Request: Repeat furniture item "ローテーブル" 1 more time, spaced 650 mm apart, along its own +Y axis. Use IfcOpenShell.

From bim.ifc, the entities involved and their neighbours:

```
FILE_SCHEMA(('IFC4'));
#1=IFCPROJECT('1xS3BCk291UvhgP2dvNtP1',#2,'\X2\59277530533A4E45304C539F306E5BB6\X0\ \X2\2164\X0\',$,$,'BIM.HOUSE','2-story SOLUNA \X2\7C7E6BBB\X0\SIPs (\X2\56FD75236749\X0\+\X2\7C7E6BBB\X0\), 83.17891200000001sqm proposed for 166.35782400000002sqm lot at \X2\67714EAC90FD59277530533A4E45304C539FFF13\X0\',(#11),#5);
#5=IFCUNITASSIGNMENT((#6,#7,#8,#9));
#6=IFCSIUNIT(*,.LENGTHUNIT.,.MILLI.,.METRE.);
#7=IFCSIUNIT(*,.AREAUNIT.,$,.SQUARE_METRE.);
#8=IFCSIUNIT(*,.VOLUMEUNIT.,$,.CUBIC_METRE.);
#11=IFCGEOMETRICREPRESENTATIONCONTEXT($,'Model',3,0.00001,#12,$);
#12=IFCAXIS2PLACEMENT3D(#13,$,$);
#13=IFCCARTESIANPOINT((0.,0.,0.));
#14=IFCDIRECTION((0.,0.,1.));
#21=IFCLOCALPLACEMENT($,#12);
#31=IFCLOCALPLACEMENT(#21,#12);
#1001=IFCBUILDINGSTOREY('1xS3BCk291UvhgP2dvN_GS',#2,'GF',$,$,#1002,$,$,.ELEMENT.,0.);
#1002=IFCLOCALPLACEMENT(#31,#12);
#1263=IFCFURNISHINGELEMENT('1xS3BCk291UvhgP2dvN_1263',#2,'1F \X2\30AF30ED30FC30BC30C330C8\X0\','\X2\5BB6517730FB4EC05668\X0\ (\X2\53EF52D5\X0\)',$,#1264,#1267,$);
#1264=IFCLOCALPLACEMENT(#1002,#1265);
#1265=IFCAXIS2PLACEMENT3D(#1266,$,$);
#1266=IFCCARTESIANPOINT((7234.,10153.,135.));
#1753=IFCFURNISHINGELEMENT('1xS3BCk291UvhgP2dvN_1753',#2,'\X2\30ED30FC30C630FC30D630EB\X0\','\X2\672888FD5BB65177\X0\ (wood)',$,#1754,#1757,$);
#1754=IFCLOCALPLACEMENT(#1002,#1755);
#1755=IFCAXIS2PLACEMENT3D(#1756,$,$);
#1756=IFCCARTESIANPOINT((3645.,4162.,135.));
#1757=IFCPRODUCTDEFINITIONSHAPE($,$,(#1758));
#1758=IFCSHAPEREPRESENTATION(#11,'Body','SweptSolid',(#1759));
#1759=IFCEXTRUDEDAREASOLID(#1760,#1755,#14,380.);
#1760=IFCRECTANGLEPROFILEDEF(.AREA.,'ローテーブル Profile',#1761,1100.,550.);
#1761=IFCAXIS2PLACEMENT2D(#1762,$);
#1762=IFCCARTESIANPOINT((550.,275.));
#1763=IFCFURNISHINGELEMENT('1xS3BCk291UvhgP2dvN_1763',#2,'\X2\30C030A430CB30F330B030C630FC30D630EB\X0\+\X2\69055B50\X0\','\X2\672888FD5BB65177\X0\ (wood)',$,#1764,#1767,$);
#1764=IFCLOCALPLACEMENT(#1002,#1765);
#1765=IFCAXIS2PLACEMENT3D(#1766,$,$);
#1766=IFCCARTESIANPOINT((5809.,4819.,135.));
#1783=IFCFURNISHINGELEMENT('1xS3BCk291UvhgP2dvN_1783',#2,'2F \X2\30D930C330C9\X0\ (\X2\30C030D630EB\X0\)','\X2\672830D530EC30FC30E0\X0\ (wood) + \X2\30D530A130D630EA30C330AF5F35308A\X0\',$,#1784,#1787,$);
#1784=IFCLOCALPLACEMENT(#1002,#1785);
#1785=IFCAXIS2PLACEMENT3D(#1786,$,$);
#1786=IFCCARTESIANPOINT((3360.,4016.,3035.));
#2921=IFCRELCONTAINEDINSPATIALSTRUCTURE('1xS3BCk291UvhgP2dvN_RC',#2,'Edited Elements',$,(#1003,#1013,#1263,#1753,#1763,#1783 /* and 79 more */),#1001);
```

```python
import ifcopenshell
import ifcopenshell.api.geometry
import ifcopenshell.api.root
import ifcopenshell.util.element
import ifcopenshell.util.placement

model = ifcopenshell.open("bim.ifc")


def reuse_history(source, copy):
    """copy_class also copies each property set's owner history, people and application; keep the originals."""
    for rel in copy.IsDefinedBy:
        if rel.is_a("IfcRelDefinesByProperties") and (history := rel.RelatingPropertyDefinition.OwnerHistory):
            rel.RelatingPropertyDefinition.OwnerHistory = source.OwnerHistory
            ifcopenshell.util.element.remove_deep2(model, history)


source = model.by_id(1753)
base = ifcopenshell.util.placement.get_local_placement(source.ObjectPlacement)
step = base[:3, 1] * 650.0

for i in range(1, 2):
    copy = ifcopenshell.api.root.copy_class(model, product=source)
    copy.Representation = ifcopenshell.util.element.copy_deep(
        model, source.Representation, exclude=["IfcGeometricRepresentationContext", "IfcRepresentationMap"]
    )
    reuse_history(source, copy)
    matrix = base.copy()
    matrix[:3, 3] += i * step
    print("added at", matrix[:3, 3].round(3) + 0.0)
    ifcopenshell.api.geometry.edit_object_placement(model, product=copy, matrix=matrix, is_si=False)

model.write("bim_v2.ifc")
```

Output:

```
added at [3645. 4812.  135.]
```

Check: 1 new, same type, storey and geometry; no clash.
